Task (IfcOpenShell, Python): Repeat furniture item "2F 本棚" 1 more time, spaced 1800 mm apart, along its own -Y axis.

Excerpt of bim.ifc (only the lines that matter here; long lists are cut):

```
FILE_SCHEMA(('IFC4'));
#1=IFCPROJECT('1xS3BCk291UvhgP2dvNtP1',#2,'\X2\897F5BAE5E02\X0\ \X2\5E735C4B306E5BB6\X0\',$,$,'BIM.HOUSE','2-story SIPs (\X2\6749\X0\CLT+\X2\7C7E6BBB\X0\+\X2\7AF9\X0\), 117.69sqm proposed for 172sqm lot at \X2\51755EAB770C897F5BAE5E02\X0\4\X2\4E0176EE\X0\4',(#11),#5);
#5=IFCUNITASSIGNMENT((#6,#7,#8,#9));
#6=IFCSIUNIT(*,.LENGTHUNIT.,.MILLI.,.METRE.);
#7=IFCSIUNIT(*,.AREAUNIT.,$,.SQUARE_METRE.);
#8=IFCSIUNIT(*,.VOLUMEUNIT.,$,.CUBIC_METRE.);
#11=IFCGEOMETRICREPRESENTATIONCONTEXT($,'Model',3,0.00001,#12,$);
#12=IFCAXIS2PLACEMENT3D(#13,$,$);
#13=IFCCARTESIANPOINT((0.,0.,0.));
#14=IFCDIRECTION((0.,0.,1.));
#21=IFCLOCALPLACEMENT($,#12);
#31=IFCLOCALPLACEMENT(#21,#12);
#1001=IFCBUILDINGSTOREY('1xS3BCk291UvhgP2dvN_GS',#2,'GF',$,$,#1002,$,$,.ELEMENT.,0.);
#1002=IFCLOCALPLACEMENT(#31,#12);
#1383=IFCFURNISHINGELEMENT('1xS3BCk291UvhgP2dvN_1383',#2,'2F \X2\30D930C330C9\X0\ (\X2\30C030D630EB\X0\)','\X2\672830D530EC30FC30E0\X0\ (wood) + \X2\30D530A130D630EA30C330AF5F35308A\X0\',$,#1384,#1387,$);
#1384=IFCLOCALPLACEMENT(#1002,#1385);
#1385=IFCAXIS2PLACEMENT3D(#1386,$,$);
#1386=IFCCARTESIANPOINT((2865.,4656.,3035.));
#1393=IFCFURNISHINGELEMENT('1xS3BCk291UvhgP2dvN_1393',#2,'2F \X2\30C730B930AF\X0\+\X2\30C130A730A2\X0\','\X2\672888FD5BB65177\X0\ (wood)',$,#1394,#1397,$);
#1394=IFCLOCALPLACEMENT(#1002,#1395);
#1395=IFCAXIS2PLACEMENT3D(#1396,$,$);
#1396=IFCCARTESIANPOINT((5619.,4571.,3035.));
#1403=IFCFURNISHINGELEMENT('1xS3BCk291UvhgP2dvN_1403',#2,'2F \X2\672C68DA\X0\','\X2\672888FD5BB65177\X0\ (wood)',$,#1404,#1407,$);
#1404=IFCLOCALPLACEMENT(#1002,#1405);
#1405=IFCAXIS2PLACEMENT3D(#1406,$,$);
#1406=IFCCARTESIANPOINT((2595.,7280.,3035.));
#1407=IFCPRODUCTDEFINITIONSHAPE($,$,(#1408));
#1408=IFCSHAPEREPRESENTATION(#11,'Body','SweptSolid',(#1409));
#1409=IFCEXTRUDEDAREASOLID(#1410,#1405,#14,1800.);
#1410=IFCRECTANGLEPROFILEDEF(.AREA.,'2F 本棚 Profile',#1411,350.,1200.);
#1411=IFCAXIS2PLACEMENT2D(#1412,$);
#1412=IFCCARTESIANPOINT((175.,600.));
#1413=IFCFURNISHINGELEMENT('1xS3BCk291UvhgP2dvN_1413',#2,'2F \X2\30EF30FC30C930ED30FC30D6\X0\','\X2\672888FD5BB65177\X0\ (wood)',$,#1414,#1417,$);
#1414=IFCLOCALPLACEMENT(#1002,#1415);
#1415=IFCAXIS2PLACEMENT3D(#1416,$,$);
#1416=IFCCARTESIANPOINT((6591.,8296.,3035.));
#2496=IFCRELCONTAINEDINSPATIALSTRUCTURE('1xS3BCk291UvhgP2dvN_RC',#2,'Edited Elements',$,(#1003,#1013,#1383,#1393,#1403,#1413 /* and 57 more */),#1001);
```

```python
import ifcopenshell
import ifcopenshell.api.geometry
import ifcopenshell.api.root
import ifcopenshell.util.element
import ifcopenshell.util.placement

model = ifcopenshell.open("bim.ifc")


def reuse_history(source, copy):
    """copy_class also copies each property set's owner history, people and application; keep the originals."""
    for rel in copy.IsDefinedBy:
        if rel.is_a("IfcRelDefinesByProperties") and (history := rel.RelatingPropertyDefinition.OwnerHistory):
            rel.RelatingPropertyDefinition.OwnerHistory = source.OwnerHistory
            ifcopenshell.util.element.remove_deep2(model, history)


source = model.by_guid("1xS3BCk291UvhgP2dvN_1403")
base = ifcopenshell.util.placement.get_local_placement(source.ObjectPlacement)
step = -base[:3, 1] * 1800.0

for i in range(1, 2):
    copy = ifcopenshell.api.root.copy_class(model, product=source)
    copy.Representation = ifcopenshell.util.element.copy_deep(
        model, source.Representation, exclude=["IfcGeometricRepresentationContext", "IfcRepresentationMap"]
    )
    reuse_history(source, copy)
    matrix = base.copy()
    matrix[:3, 3] += i * step
    print("added at", matrix[:3, 3].round(3) + 0.0)
    ifcopenshell.api.geometry.edit_object_placement(model, product=copy, matrix=matrix, is_si=False)

model.write("bim_updated.ifc")
```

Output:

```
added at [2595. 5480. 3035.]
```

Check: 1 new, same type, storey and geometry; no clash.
